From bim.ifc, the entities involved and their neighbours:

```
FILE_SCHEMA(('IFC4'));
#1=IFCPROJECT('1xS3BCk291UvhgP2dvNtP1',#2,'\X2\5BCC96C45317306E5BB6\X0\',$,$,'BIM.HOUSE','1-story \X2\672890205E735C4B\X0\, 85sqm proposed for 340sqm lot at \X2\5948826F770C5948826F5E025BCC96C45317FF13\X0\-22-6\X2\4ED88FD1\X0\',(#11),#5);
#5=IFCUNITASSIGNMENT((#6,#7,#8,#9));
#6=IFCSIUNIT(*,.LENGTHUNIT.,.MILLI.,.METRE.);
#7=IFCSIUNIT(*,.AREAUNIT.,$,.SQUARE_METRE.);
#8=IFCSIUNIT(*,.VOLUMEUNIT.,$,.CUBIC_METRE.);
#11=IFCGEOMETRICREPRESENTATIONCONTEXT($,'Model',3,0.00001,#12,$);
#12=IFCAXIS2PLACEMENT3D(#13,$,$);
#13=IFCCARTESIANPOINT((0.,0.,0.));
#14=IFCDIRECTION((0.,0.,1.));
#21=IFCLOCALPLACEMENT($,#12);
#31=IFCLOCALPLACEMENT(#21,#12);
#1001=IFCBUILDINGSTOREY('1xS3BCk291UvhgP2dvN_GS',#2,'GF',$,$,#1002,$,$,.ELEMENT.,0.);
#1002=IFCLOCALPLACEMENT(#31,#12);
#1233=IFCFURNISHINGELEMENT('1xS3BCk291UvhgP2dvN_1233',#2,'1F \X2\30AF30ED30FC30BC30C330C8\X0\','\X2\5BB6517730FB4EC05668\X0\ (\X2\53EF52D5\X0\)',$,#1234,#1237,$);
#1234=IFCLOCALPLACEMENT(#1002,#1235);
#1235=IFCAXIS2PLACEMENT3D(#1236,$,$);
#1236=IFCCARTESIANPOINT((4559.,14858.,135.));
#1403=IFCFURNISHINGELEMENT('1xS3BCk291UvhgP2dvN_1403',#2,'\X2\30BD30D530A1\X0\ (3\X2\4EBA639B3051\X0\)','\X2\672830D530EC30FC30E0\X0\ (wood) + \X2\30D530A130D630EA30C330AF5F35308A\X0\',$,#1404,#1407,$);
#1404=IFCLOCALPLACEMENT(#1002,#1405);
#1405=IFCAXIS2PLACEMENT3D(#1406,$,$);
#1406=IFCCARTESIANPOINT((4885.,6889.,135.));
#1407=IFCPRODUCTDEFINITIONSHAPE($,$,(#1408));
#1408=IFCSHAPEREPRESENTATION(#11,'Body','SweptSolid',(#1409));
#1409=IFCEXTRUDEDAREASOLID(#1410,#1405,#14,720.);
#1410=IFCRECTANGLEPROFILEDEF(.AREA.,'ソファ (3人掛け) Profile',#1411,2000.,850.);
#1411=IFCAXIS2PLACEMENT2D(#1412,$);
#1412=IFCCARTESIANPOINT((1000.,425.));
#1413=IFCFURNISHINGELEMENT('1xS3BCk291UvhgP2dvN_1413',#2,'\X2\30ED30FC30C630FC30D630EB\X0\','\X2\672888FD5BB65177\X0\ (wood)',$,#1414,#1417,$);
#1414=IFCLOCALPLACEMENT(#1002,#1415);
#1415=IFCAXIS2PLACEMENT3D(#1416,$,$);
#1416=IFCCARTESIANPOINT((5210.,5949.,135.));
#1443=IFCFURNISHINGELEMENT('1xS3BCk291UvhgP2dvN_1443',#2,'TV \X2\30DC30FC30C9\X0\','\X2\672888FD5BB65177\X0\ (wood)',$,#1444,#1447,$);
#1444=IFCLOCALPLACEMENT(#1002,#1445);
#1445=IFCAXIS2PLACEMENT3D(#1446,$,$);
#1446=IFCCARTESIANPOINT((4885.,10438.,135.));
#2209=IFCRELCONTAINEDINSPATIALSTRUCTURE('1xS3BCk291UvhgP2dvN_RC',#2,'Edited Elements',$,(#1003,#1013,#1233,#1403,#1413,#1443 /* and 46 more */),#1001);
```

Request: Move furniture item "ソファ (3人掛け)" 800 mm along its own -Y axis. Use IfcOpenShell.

```python
import ifcopenshell
import ifcopenshell.api.geometry
import ifcopenshell.util.placement
import ifcopenshell.util.unit

model = ifcopenshell.open("bim.ifc")
unit_scale = ifcopenshell.util.unit.calculate_unit_scale(model)

item = model.by_id(1403)
matrix = ifcopenshell.util.placement.get_local_placement(item.ObjectPlacement)
matrix[:3, 3] -= matrix[:3, 1] * 0.8 / unit_scale
ifcopenshell.api.geometry.edit_object_placement(model, product=item, matrix=matrix, is_si=False)

print(ifcopenshell.util.placement.get_local_placement(item.ObjectPlacement).round(3) + 0.0)

model.write("bim_rev.ifc")
```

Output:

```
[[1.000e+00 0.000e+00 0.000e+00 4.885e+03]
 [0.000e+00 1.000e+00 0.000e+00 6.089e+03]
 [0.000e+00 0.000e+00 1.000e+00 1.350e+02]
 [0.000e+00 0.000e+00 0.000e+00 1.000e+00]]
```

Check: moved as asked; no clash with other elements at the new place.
